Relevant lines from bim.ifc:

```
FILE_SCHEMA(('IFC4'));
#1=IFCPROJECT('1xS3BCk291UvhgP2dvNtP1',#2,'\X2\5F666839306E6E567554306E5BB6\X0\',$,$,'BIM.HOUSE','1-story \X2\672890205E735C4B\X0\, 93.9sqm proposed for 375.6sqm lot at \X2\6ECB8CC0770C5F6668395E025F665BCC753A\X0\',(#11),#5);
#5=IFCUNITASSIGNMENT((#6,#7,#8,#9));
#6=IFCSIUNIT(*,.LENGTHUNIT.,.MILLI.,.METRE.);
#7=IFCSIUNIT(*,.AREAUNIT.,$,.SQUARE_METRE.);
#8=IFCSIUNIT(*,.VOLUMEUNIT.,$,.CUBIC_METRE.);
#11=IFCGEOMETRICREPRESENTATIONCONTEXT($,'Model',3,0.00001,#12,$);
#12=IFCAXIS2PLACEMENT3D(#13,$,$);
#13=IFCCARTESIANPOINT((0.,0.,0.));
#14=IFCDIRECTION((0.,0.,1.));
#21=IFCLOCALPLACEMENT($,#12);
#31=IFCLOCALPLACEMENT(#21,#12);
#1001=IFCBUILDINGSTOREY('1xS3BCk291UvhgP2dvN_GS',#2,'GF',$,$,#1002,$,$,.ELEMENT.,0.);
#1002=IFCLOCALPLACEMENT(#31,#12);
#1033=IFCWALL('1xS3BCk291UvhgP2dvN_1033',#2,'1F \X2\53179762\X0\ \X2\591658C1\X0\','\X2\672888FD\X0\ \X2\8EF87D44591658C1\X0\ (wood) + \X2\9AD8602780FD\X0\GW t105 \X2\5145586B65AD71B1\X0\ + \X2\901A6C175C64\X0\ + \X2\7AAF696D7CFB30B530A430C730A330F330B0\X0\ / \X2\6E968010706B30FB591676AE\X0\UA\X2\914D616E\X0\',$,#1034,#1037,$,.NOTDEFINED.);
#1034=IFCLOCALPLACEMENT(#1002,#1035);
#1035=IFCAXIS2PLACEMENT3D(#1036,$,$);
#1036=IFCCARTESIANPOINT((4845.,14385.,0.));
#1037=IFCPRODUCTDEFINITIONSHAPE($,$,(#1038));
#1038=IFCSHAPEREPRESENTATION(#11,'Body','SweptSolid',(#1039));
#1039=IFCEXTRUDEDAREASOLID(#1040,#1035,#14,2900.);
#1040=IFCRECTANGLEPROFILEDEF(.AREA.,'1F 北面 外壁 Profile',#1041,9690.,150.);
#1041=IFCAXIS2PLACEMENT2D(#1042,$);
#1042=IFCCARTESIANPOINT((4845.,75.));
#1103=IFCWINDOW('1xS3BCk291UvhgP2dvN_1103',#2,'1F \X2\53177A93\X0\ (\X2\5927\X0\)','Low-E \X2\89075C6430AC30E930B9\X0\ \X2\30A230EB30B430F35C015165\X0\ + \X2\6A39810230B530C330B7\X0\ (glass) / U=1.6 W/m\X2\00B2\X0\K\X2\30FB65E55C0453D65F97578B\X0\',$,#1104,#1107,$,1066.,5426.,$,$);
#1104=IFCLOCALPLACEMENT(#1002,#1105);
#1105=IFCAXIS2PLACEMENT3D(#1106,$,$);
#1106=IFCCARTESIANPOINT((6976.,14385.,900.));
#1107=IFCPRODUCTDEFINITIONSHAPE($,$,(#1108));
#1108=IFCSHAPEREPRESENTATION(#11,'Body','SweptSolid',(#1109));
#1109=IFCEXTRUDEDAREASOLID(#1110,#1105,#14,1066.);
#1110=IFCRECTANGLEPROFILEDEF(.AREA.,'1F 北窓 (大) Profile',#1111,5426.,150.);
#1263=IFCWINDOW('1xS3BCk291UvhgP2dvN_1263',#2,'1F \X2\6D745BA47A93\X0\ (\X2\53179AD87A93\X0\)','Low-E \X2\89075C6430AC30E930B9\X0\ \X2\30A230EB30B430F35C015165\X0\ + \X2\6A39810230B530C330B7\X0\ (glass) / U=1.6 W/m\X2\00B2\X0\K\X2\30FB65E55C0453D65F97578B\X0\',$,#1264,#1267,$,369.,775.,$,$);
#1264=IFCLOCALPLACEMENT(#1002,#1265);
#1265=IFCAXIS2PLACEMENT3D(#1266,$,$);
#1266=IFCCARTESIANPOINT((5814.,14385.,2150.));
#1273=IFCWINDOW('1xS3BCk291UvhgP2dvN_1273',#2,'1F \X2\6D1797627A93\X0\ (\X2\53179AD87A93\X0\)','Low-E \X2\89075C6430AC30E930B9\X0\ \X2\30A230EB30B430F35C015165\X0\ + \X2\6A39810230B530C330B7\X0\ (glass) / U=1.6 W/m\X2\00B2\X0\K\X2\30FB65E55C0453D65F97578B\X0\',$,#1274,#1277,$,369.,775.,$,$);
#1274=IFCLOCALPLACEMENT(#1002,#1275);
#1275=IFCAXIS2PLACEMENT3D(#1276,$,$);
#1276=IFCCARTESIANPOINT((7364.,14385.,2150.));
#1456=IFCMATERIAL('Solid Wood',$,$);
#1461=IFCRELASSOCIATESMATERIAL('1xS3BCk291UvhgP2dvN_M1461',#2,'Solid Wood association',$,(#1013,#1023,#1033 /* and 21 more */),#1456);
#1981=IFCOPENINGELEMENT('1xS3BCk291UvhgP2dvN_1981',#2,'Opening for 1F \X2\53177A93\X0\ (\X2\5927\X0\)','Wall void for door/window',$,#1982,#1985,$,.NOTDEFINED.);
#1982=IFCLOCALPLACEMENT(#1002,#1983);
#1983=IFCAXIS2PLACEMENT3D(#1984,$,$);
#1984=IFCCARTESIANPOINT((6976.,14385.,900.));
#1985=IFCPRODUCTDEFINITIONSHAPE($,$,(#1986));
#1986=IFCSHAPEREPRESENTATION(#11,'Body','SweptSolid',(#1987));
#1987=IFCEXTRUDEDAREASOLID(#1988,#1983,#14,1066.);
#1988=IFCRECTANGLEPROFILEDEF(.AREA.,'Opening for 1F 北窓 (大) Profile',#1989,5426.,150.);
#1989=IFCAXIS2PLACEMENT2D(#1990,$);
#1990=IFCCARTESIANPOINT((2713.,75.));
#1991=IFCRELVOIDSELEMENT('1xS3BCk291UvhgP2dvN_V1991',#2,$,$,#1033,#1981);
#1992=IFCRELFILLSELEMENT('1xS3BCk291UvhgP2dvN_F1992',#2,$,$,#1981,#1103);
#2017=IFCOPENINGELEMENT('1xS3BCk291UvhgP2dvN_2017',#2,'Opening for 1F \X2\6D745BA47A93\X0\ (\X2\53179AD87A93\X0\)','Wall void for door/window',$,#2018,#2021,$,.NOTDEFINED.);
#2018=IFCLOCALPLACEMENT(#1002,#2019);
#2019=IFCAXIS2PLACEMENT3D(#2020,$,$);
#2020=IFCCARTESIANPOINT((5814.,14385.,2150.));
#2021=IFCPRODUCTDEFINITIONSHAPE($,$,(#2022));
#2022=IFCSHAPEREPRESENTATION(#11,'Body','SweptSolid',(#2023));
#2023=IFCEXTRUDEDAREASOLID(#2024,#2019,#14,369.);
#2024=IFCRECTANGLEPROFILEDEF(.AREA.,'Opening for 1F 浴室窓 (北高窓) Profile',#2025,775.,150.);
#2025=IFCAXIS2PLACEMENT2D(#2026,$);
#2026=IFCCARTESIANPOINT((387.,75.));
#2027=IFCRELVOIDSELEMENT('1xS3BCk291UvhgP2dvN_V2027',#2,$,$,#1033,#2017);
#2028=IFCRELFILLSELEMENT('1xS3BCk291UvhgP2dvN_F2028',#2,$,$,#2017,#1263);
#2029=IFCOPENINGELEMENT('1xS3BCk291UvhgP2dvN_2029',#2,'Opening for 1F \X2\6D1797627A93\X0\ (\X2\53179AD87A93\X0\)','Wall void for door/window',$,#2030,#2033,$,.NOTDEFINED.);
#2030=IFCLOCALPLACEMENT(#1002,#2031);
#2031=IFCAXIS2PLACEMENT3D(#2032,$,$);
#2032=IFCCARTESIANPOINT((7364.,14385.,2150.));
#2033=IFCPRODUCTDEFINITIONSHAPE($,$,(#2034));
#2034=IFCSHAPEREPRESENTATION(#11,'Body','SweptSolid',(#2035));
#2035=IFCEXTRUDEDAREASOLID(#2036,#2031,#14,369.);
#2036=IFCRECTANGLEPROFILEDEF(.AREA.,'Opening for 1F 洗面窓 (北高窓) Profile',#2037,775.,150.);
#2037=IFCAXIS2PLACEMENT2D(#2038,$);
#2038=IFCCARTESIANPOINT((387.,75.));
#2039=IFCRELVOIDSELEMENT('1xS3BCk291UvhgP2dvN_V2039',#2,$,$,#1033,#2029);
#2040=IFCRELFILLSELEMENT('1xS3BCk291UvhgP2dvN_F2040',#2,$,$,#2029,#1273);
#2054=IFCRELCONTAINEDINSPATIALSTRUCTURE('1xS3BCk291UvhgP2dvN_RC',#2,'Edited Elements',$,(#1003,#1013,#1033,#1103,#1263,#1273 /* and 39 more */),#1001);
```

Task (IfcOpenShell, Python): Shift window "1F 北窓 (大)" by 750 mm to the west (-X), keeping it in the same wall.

```python
import ifcopenshell
import ifcopenshell.api.geometry
import ifcopenshell.util.placement
import ifcopenshell.util.unit

model = ifcopenshell.open("bim.ifc")
unit_scale = ifcopenshell.util.unit.calculate_unit_scale(model)

window = model.by_id(1103)
opening = window.FillsVoids[0].RelatingOpeningElement
wall = opening.VoidsElements[0].RelatingBuildingElement

wall_matrix = ifcopenshell.util.placement.get_local_placement(wall.ObjectPlacement)
shift = wall_matrix[:3, 0] * -0.75 / unit_scale
before = ifcopenshell.util.placement.get_local_placement(window.ObjectPlacement)[:3, 3].copy()

# The window is not placed relative to its opening, so move both.
for product in (opening, window):
    matrix = ifcopenshell.util.placement.get_local_placement(product.ObjectPlacement)
    matrix[:3, 3] += shift
    ifcopenshell.api.geometry.edit_object_placement(model, product=product, matrix=matrix, is_si=False)

after = ifcopenshell.util.placement.get_local_placement(window.ObjectPlacement)[:3, 3]
print("window moved by", (after - before).round(3) + 0.0)

model.write("bim-out.ifc")
```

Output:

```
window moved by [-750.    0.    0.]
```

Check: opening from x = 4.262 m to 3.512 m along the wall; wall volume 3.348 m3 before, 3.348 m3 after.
